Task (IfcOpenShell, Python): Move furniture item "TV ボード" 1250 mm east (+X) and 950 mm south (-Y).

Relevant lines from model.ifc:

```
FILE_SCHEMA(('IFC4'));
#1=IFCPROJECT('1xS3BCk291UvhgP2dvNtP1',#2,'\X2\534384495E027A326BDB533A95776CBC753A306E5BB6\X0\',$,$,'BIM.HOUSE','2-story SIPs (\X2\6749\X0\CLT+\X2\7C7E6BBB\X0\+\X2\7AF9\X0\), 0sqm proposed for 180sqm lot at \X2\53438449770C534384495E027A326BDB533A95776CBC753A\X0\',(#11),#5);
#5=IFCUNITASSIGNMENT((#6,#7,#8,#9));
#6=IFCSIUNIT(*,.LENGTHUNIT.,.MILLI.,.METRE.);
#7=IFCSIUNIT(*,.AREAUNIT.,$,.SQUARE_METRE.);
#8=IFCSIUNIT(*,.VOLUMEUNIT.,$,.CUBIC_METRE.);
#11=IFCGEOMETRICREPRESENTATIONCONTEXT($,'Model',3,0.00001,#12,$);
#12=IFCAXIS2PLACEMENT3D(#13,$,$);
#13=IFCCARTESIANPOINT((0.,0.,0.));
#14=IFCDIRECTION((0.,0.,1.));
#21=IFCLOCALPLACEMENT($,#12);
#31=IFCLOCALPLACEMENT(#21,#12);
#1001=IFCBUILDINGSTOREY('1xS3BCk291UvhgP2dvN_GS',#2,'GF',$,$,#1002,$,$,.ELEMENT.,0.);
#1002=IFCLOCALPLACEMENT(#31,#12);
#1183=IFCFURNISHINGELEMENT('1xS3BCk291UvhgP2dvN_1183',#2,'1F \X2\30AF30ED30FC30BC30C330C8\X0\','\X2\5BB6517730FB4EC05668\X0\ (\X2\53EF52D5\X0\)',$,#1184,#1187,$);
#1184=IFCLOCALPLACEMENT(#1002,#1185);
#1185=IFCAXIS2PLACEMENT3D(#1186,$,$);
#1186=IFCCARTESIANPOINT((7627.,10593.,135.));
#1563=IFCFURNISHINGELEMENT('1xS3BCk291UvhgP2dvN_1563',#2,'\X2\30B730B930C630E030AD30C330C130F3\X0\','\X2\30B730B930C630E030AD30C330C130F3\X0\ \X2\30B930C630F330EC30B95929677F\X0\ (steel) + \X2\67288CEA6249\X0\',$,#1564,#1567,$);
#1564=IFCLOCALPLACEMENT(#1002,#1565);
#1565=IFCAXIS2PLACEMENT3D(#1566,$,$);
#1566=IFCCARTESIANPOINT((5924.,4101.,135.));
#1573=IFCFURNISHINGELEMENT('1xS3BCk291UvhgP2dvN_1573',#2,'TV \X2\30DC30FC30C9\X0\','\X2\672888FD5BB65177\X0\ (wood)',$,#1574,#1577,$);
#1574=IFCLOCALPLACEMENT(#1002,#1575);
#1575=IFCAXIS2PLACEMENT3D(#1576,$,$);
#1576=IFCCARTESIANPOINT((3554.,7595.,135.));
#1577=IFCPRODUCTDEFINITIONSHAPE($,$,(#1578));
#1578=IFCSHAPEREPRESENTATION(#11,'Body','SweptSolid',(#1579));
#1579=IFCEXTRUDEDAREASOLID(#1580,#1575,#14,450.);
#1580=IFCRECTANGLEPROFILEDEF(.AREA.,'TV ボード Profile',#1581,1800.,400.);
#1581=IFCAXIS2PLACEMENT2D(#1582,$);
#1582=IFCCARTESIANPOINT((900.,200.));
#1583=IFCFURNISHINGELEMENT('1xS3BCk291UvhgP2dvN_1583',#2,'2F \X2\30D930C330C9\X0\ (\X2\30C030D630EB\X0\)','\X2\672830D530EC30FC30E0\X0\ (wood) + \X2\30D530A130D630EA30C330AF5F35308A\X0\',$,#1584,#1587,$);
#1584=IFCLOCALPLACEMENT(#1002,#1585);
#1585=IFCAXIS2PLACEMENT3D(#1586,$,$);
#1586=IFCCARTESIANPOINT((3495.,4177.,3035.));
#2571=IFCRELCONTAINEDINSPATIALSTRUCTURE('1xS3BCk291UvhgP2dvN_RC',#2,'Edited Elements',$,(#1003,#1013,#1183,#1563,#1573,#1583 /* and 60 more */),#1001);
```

```python
import ifcopenshell
import ifcopenshell.api.geometry
import ifcopenshell.util.placement

model = ifcopenshell.open("model.ifc")

item = model.by_guid("1xS3BCk291UvhgP2dvN_1573")
matrix = ifcopenshell.util.placement.get_local_placement(item.ObjectPlacement)
matrix[0, 3] += 1250.0
matrix[1, 3] -= 950.0
ifcopenshell.api.geometry.edit_object_placement(model, product=item, matrix=matrix, is_si=False)

print(ifcopenshell.util.placement.get_local_placement(item.ObjectPlacement).round(3) + 0.0)

model.write("model_edited.ifc")
```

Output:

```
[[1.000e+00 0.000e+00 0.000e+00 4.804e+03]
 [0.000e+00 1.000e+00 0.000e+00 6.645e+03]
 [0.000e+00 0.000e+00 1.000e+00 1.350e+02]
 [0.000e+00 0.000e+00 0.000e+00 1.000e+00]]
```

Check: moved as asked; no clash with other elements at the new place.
